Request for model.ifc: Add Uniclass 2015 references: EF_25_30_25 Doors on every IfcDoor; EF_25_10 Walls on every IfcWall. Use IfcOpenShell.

First a look at what the model holds.

```python
import ifcopenshell

model = ifcopenshell.open("model.ifc")
print(model.schema)
print("classifications:", [c.Name for c in model.by_type("IfcClassification")])
for ifc_class in ("IfcDoor", "IfcRoof", "IfcStair", "IfcWall", "IfcWindow"):
    print(ifc_class, len(model.by_type(ifc_class)))
```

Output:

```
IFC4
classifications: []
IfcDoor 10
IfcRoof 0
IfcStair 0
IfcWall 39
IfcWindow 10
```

```python
import ifcopenshell
import ifcopenshell.api.classification

model = ifcopenshell.open("model.ifc")

system = ifcopenshell.api.classification.add_classification(model, classification="Uniclass 2015")

codes = {
    "IfcDoor": ("EF_25_30_25", "Doors"),
    "IfcWall": ("EF_25_10", "Walls"),
}
for ifc_class, (code, name) in codes.items():
    products = model.by_type(ifc_class)
    ifcopenshell.api.classification.add_reference(
        model, products=products, classification=system, identification=code, name=name
    )
    print(code, len(products))

model.write("model_edited.ifc")
```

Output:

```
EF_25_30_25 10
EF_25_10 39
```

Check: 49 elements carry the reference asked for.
